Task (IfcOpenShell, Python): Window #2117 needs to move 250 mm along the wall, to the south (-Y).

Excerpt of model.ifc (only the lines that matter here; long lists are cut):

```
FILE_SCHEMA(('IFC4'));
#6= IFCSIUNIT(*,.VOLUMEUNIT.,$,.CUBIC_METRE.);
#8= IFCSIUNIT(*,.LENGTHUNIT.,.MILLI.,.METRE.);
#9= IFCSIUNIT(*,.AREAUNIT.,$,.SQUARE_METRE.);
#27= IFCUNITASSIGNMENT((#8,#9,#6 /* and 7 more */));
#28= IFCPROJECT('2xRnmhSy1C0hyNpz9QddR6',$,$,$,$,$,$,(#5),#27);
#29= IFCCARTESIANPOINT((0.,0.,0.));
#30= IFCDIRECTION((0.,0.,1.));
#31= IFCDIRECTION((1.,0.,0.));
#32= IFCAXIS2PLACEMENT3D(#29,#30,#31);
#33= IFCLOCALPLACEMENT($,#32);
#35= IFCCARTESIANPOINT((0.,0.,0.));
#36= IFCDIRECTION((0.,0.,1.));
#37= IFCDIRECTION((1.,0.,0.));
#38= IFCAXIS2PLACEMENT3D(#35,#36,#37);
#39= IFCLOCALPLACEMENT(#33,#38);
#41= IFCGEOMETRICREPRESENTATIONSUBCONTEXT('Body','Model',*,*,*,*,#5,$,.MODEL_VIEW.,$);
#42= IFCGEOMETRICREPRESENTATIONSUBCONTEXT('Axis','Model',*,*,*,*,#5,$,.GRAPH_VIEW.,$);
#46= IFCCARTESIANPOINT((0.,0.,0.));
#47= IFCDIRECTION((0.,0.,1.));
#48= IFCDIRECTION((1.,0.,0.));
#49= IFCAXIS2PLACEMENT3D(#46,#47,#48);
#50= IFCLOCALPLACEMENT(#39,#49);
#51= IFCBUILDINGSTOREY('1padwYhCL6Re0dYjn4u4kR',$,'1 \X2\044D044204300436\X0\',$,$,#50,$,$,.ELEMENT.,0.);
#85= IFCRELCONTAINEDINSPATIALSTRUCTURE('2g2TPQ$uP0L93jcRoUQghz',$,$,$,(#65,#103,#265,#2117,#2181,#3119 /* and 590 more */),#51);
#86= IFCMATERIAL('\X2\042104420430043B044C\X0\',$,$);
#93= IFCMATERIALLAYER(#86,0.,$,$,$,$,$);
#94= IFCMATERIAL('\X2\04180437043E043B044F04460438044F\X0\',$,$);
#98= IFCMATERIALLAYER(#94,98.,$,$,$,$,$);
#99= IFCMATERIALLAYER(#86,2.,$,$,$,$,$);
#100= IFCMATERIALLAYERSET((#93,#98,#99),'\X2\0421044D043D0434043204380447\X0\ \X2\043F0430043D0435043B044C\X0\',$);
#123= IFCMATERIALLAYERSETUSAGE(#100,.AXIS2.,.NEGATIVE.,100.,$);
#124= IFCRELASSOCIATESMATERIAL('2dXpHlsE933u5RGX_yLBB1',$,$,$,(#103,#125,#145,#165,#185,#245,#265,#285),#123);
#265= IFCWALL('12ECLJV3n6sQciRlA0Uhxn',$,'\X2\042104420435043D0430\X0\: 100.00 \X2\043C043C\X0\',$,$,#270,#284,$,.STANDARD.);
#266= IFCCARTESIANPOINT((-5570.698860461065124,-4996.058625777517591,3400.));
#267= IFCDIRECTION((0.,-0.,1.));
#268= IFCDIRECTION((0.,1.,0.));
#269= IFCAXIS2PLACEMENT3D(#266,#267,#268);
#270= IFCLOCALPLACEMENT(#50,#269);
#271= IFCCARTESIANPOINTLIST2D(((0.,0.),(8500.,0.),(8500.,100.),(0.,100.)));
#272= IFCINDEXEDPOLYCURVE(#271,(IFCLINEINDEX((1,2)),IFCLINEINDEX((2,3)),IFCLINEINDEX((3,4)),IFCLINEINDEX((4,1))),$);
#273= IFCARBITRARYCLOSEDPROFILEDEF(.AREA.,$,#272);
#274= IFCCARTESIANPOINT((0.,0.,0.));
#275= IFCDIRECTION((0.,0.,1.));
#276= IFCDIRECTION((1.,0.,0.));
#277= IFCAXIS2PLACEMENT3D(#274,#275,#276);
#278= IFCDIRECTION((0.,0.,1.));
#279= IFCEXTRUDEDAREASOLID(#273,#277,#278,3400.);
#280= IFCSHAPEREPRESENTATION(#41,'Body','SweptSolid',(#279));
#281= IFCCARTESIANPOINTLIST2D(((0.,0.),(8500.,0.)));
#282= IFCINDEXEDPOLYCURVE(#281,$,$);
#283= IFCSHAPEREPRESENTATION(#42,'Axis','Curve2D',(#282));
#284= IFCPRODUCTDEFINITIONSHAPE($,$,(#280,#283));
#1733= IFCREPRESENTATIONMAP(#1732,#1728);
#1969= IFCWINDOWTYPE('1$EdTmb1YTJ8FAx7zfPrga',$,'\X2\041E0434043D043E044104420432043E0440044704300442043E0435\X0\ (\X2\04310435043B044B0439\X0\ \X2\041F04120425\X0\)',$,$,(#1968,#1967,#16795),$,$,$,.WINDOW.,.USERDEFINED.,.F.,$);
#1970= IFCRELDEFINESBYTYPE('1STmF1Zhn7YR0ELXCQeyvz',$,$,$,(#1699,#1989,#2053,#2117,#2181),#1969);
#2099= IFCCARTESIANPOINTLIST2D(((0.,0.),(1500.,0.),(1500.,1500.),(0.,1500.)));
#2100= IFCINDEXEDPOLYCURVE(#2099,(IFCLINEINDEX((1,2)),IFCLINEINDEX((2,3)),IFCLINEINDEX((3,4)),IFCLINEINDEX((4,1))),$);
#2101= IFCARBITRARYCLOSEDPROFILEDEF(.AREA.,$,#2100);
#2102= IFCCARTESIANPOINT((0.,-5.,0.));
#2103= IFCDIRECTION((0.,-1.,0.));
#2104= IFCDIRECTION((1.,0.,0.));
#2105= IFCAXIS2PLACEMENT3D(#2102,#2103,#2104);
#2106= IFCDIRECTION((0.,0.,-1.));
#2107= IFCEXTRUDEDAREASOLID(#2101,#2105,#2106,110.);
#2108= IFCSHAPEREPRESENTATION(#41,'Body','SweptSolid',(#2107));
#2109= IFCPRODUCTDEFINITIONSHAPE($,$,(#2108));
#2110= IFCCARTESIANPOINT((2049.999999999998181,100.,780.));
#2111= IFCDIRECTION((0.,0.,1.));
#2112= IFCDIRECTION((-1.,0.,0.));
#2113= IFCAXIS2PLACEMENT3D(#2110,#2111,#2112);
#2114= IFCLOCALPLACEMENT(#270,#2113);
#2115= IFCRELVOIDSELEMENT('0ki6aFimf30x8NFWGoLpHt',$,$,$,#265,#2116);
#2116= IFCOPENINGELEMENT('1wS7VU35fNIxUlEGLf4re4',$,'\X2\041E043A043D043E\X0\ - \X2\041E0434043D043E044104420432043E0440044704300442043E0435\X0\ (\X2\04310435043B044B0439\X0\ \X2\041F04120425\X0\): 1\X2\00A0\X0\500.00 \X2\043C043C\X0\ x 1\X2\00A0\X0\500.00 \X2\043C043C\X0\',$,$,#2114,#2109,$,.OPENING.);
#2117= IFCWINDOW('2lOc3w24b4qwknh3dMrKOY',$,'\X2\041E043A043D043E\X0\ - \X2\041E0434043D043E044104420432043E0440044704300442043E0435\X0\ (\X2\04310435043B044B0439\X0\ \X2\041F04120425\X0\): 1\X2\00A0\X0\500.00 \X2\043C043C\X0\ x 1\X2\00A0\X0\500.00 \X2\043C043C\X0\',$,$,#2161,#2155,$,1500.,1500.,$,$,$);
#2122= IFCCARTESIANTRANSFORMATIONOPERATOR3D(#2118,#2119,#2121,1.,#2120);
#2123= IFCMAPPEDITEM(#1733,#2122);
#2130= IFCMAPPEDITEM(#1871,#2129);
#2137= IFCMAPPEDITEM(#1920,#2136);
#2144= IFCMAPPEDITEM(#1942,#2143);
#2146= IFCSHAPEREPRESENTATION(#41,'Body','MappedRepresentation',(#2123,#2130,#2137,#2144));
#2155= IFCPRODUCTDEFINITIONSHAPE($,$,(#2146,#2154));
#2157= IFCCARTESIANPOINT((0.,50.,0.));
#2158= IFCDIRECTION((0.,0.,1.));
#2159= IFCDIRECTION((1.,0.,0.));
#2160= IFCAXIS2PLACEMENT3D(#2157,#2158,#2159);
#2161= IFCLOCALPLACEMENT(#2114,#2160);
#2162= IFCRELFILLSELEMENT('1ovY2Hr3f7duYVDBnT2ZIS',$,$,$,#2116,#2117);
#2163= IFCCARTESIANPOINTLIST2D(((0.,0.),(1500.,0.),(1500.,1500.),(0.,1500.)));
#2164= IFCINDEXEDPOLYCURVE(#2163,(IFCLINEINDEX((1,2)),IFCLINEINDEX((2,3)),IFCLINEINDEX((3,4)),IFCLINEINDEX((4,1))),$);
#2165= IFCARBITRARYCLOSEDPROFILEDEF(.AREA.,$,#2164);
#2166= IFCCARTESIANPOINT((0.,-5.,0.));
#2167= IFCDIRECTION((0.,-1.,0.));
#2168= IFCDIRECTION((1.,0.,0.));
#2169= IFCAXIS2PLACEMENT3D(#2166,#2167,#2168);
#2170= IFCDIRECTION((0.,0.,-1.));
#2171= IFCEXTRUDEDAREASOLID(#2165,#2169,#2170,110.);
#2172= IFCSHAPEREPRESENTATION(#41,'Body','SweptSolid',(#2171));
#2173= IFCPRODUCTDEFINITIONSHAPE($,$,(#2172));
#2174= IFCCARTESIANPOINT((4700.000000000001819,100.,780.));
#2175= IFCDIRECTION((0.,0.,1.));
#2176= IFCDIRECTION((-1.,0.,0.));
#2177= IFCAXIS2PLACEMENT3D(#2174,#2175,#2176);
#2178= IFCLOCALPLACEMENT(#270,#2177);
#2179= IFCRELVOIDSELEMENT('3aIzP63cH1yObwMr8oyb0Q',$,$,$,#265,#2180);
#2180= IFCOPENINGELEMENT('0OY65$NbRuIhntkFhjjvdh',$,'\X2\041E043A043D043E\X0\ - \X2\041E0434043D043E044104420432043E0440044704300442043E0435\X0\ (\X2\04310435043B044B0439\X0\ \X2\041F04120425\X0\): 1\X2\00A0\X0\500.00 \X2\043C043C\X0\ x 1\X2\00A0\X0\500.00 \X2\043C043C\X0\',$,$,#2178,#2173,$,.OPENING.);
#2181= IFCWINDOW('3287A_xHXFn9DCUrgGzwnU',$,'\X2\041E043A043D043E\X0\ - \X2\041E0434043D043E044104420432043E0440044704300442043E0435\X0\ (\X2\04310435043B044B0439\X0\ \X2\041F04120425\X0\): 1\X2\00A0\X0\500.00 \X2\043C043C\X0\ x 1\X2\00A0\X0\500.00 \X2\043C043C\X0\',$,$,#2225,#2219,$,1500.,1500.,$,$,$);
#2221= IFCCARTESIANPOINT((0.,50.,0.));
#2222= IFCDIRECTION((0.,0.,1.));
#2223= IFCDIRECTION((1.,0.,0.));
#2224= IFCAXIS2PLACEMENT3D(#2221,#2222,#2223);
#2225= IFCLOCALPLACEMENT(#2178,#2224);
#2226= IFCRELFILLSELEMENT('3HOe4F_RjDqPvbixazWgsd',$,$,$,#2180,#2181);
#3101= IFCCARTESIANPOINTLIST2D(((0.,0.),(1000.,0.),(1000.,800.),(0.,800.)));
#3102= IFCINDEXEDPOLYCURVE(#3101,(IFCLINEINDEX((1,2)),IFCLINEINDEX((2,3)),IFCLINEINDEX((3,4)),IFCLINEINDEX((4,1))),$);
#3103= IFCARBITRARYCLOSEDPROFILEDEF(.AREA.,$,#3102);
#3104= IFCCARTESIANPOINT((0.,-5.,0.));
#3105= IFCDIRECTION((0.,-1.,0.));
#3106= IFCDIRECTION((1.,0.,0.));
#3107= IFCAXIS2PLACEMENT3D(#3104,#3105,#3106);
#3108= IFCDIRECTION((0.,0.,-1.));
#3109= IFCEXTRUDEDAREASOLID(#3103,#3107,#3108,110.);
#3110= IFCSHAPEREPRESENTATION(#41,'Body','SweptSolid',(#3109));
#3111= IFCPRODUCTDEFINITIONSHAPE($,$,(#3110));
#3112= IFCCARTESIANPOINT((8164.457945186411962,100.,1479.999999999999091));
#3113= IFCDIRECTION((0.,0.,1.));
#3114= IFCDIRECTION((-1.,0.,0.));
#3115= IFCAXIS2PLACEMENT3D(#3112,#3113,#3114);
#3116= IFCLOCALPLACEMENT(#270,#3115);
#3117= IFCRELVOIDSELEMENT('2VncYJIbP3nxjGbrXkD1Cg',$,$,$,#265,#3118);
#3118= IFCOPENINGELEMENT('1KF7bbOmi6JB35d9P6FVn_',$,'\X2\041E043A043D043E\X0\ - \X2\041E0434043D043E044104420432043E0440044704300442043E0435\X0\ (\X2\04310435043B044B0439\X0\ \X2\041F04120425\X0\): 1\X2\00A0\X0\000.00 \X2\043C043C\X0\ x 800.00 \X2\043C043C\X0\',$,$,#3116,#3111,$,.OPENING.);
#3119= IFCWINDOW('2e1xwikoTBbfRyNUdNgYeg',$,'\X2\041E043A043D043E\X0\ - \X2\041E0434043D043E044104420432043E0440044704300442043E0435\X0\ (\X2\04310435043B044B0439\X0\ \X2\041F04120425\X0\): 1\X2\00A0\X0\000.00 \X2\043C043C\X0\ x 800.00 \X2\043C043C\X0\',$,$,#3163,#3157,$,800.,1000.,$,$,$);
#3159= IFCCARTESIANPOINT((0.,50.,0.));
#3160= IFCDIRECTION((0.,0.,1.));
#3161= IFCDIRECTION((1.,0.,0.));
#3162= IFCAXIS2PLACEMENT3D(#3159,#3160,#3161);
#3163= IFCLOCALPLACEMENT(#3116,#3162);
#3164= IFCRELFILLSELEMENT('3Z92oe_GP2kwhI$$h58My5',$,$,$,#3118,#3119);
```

```python
import ifcopenshell
import ifcopenshell.api.geometry
import ifcopenshell.util.placement
import ifcopenshell.util.unit

model = ifcopenshell.open("model.ifc")
unit_scale = ifcopenshell.util.unit.calculate_unit_scale(model)

window = model.by_id(2117)
opening = window.FillsVoids[0].RelatingOpeningElement
wall = opening.VoidsElements[0].RelatingBuildingElement

wall_matrix = ifcopenshell.util.placement.get_local_placement(wall.ObjectPlacement)
shift = wall_matrix[:3, 0] * -0.25 / unit_scale
before = ifcopenshell.util.placement.get_local_placement(window.ObjectPlacement)[:3, 3].copy()

# The window is placed relative to its opening, so it follows when the opening moves.
matrix = ifcopenshell.util.placement.get_local_placement(opening.ObjectPlacement)
matrix[:3, 3] += shift
ifcopenshell.api.geometry.edit_object_placement(
    model, product=opening, matrix=matrix, is_si=False, should_transform_children=True
)

after = ifcopenshell.util.placement.get_local_placement(window.ObjectPlacement)[:3, 3]
print("window moved by", (after - before).round(3) + 0.0)

model.write("model_v2.ifc")
```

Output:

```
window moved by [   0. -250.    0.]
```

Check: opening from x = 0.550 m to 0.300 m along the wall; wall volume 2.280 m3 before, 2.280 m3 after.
